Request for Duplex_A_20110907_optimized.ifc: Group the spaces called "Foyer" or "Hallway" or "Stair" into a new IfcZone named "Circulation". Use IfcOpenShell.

First a look at what the model holds.

```python
import ifcopenshell

model = ifcopenshell.open("Duplex_A_20110907_optimized.ifc")
print(model.schema)
seen = {}
for space in model.by_type("IfcSpace"):
    seen[space.LongName] = seen.get(space.LongName, 0) + 1
for name, count in sorted(seen.items(), key=str):
    print(count, "x", name)
print("zones:", [z.Name for z in model.by_type("IfcZone")][:20])
```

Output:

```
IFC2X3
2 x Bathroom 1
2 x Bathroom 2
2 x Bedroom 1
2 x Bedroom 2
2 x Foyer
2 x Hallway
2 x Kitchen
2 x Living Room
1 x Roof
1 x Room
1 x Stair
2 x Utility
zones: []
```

```python
import ifcopenshell
import ifcopenshell.api.group
import ifcopenshell.api.root

model = ifcopenshell.open("Duplex_A_20110907_optimized.ifc")

names = {"Foyer", "Hallway", "Stair"}
spaces = [s for s in model.by_type("IfcSpace") if s.LongName in names]

zone = ifcopenshell.api.root.create_entity(model, ifc_class="IfcZone", name="Circulation")
ifcopenshell.api.group.assign_group(model, products=spaces, group=zone)
print(len(spaces), "spaces in", zone.Name)

model.write("Duplex_A_20110907_optimized_rev.ifc")
```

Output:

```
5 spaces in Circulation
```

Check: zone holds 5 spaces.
